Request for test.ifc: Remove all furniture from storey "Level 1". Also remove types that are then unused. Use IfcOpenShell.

First a look at what the model holds.

```python
import ifcopenshell
import ifcopenshell.util.element

model = ifcopenshell.open("test.ifc")
print(model.schema)
storey = next(s for s in model.by_type("IfcBuildingStorey") if s.Name == "Level 1")
furniture = [e for e in ifcopenshell.util.element.get_decomposition(storey) if e.is_a("IfcFurnishingElement")]
seen = {}
for e in furniture:
    element_type = ifcopenshell.util.element.get_type(e)
    name = element_type.Name if element_type not in (None, e) else None
    seen[name] = seen.get(name, 0) + 1
for name, count in sorted(seen.items(), key=str):
    print(count, "x", name)
```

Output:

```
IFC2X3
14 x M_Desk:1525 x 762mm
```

```python
import ifcopenshell
import ifcopenshell.api.root
import ifcopenshell.util.element

model = ifcopenshell.open("test.ifc")

storey = next(s for s in model.by_type("IfcBuildingStorey") if s.Name == "Level 1")
furniture = [e for e in ifcopenshell.util.element.get_decomposition(storey) if e.is_a("IfcFurnishingElement")]
types = {ifcopenshell.util.element.get_type(e) for e in furniture} - {None, *furniture}

for e in furniture:
    ifcopenshell.api.root.remove_product(model, product=e)
print(len(furniture), "removed")

unused = [t for t in types if not ifcopenshell.util.element.get_types(t)]
for t in unused:
    ifcopenshell.api.root.remove_product(model, product=t)
print(len(unused), "unused types removed")

model.write("test-out.ifc")
```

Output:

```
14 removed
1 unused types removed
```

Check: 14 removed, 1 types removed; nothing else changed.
